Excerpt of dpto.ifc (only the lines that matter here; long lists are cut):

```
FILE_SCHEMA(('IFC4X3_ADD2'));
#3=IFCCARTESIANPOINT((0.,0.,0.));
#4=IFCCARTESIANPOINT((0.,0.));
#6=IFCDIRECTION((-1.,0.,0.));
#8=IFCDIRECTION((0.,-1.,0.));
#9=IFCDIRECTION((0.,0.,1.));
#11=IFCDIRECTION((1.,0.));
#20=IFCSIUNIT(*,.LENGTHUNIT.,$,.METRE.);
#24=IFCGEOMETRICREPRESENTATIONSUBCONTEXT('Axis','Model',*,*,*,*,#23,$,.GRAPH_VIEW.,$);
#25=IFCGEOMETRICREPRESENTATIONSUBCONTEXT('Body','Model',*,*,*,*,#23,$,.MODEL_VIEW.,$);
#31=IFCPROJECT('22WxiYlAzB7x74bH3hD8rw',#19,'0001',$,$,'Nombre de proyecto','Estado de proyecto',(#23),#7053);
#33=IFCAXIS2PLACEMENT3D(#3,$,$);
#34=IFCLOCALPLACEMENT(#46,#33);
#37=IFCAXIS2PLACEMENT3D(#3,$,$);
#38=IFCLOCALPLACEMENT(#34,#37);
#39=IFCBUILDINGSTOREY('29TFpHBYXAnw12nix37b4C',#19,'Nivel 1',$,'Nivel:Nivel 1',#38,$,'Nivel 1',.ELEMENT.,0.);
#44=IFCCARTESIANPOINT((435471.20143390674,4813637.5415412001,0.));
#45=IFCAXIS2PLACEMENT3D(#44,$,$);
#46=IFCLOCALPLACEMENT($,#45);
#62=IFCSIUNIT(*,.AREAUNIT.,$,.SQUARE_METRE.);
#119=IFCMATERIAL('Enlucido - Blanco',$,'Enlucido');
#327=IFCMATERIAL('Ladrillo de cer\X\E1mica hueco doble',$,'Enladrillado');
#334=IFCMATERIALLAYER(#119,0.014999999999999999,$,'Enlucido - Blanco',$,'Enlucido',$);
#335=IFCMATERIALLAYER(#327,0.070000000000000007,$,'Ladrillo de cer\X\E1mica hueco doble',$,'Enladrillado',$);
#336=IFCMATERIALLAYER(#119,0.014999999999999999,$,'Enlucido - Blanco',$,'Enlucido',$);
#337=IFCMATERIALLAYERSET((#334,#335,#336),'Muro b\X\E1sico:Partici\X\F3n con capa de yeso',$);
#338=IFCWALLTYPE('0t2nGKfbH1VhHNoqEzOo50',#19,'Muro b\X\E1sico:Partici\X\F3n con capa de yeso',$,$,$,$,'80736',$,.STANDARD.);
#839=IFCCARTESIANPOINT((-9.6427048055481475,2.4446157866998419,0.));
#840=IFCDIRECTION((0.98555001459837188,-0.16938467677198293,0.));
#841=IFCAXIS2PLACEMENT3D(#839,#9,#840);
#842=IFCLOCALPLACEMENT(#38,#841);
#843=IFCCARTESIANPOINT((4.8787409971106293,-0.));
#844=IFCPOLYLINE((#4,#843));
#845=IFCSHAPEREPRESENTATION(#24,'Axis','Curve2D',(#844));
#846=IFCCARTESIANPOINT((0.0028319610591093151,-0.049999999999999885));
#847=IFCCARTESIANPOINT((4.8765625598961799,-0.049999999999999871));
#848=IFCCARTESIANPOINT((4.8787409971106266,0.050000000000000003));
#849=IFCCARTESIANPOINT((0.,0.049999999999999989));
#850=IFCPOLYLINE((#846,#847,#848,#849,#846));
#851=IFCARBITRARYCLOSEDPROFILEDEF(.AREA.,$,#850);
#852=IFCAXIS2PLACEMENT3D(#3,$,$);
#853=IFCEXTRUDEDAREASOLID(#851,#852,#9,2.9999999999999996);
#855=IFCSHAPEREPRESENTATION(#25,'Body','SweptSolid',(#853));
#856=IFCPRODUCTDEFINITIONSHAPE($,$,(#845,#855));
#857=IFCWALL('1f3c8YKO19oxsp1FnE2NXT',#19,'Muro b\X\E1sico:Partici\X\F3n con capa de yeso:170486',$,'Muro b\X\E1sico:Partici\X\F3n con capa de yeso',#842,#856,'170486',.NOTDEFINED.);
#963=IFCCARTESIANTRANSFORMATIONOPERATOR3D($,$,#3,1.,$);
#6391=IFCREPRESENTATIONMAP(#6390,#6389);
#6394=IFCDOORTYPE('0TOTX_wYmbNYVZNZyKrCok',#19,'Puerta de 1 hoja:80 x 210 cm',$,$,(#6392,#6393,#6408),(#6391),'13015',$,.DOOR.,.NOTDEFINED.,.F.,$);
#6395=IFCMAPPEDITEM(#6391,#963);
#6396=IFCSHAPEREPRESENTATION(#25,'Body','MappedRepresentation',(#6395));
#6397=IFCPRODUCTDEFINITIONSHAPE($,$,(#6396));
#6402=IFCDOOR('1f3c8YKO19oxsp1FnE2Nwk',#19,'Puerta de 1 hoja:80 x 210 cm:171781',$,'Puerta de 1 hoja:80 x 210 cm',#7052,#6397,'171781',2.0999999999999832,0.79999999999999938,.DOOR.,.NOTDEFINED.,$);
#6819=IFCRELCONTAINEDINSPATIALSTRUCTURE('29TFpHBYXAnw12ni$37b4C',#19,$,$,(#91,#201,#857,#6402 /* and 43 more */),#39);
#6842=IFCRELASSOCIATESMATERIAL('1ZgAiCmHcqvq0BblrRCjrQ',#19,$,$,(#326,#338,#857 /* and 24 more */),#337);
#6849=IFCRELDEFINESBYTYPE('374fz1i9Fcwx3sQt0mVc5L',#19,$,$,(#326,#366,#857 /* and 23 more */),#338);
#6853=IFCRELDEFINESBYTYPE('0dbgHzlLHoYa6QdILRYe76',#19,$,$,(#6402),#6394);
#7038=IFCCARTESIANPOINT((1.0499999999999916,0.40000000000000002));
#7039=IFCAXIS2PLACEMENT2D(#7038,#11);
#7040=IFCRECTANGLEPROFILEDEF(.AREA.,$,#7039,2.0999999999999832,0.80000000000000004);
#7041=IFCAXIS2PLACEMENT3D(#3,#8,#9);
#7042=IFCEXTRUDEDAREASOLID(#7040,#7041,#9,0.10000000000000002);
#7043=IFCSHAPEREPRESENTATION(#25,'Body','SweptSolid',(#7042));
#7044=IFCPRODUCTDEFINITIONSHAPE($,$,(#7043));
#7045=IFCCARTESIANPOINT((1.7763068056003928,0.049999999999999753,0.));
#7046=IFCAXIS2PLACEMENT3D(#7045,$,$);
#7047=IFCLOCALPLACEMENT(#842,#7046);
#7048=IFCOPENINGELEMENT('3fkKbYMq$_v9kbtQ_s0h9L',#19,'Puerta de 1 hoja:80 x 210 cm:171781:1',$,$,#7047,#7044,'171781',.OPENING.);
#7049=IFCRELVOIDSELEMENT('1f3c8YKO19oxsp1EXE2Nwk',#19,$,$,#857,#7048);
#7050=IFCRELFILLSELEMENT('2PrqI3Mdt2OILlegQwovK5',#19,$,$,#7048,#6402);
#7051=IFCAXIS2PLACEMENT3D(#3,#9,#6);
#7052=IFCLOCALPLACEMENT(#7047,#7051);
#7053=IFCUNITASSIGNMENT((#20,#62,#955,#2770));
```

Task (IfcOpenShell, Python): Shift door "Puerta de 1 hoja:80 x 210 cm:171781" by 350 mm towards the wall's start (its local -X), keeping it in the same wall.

```python
import ifcopenshell
import ifcopenshell.api.geometry
import ifcopenshell.util.placement
import ifcopenshell.util.unit

model = ifcopenshell.open("dpto.ifc")
unit_scale = ifcopenshell.util.unit.calculate_unit_scale(model)

door = model.by_id(6402)
opening = door.FillsVoids[0].RelatingOpeningElement
wall = opening.VoidsElements[0].RelatingBuildingElement

wall_matrix = ifcopenshell.util.placement.get_local_placement(wall.ObjectPlacement)
shift = wall_matrix[:3, 0] * -0.35 / unit_scale
before = ifcopenshell.util.placement.get_local_placement(door.ObjectPlacement)[:3, 3].copy()

# The door is placed relative to its opening, so it follows when the opening moves.
matrix = ifcopenshell.util.placement.get_local_placement(opening.ObjectPlacement)
matrix[:3, 3] += shift
ifcopenshell.api.geometry.edit_object_placement(
    model, product=opening, matrix=matrix, is_si=False, should_transform_children=True
)

after = ifcopenshell.util.placement.get_local_placement(door.ObjectPlacement)[:3, 3]
print("door moved by", (after - before).round(3) + 0.0)

model.write("dpto_rev.ifc")
```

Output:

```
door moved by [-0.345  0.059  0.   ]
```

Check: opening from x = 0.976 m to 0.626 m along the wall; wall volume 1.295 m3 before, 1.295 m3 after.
